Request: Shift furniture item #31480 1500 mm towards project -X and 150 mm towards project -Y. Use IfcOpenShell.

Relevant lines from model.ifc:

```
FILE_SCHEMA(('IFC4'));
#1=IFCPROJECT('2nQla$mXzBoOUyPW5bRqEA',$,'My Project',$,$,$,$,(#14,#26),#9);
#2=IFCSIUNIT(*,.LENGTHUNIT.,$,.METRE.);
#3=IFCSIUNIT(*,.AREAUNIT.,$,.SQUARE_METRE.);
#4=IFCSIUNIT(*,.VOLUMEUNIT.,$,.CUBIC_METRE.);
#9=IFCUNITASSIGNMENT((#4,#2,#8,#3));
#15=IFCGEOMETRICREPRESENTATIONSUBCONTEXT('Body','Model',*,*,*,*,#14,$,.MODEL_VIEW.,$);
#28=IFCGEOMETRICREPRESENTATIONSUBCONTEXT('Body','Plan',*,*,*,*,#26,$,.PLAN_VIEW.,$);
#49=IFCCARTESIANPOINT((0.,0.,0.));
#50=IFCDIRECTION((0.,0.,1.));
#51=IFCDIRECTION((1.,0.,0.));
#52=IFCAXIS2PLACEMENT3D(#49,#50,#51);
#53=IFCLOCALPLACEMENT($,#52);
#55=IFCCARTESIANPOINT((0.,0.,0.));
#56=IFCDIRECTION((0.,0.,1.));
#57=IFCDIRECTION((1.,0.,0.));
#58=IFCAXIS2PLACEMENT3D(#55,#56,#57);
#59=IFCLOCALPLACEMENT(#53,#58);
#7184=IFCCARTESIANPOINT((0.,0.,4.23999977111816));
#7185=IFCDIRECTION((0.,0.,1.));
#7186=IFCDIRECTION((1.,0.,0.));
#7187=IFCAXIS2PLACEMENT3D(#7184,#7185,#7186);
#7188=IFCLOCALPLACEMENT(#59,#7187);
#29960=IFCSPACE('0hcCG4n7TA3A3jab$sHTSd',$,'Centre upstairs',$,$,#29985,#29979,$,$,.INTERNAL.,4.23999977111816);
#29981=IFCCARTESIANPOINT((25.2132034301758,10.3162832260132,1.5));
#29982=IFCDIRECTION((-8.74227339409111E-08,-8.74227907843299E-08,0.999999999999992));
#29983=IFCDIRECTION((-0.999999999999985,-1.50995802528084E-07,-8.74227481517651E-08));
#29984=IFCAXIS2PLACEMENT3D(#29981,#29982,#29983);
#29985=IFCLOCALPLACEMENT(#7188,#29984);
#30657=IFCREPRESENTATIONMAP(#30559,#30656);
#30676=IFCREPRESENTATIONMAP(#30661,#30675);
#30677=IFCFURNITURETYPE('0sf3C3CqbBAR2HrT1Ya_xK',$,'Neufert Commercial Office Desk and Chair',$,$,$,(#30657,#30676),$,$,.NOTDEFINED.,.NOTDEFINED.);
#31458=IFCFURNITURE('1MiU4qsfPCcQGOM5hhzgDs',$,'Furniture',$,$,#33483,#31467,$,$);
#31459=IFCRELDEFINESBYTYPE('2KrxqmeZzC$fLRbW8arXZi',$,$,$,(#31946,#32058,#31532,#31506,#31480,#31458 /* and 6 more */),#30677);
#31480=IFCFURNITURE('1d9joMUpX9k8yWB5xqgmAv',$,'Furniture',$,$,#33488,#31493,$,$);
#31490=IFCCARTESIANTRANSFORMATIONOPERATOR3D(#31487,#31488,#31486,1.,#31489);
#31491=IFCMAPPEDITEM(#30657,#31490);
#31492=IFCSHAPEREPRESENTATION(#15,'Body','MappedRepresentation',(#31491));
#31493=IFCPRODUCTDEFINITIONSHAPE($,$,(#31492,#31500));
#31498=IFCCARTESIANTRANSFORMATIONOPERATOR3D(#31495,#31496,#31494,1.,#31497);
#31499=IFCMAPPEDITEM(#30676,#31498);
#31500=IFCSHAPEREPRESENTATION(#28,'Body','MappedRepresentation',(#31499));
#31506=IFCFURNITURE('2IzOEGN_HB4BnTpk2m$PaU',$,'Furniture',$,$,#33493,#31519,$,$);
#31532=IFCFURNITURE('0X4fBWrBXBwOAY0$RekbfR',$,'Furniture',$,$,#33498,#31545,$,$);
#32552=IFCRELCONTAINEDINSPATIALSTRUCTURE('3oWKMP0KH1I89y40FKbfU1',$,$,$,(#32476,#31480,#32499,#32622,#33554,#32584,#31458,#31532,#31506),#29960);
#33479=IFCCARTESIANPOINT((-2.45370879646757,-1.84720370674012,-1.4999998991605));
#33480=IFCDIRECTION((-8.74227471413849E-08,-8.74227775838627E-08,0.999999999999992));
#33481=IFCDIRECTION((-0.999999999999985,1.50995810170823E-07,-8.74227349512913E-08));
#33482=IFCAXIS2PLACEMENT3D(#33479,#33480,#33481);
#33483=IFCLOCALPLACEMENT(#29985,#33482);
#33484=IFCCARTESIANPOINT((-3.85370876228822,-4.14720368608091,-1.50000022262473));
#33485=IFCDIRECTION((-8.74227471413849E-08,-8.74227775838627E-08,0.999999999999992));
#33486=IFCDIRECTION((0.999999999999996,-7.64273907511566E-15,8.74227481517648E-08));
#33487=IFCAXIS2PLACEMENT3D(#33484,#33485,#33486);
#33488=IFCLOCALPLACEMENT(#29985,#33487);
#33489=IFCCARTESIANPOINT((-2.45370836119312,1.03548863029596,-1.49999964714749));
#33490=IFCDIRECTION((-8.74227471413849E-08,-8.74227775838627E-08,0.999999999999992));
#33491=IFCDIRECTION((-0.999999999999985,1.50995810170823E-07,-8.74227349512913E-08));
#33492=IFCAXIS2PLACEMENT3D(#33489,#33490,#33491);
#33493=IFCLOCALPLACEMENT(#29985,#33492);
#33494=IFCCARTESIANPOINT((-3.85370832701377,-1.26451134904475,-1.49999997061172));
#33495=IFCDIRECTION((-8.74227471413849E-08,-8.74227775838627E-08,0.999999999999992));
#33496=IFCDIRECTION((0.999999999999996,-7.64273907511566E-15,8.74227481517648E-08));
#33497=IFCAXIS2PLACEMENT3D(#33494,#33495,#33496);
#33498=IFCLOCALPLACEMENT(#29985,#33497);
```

```python
import ifcopenshell
import ifcopenshell.api.geometry
import ifcopenshell.util.placement

model = ifcopenshell.open("model.ifc")

item = model.by_guid("1d9joMUpX9k8yWB5xqgmAv")
matrix = ifcopenshell.util.placement.get_local_placement(item.ObjectPlacement)
matrix[0, 3] -= 1.5
matrix[1, 3] -= 0.15
ifcopenshell.api.geometry.edit_object_placement(model, product=item, matrix=matrix, is_si=False)

print(ifcopenshell.util.placement.get_local_placement(item.ObjectPlacement).round(3) + 0.0)

model.write("model_edited.ifc")
```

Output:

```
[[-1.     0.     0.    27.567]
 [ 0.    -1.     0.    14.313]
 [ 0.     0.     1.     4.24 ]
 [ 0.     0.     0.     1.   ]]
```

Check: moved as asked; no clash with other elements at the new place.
